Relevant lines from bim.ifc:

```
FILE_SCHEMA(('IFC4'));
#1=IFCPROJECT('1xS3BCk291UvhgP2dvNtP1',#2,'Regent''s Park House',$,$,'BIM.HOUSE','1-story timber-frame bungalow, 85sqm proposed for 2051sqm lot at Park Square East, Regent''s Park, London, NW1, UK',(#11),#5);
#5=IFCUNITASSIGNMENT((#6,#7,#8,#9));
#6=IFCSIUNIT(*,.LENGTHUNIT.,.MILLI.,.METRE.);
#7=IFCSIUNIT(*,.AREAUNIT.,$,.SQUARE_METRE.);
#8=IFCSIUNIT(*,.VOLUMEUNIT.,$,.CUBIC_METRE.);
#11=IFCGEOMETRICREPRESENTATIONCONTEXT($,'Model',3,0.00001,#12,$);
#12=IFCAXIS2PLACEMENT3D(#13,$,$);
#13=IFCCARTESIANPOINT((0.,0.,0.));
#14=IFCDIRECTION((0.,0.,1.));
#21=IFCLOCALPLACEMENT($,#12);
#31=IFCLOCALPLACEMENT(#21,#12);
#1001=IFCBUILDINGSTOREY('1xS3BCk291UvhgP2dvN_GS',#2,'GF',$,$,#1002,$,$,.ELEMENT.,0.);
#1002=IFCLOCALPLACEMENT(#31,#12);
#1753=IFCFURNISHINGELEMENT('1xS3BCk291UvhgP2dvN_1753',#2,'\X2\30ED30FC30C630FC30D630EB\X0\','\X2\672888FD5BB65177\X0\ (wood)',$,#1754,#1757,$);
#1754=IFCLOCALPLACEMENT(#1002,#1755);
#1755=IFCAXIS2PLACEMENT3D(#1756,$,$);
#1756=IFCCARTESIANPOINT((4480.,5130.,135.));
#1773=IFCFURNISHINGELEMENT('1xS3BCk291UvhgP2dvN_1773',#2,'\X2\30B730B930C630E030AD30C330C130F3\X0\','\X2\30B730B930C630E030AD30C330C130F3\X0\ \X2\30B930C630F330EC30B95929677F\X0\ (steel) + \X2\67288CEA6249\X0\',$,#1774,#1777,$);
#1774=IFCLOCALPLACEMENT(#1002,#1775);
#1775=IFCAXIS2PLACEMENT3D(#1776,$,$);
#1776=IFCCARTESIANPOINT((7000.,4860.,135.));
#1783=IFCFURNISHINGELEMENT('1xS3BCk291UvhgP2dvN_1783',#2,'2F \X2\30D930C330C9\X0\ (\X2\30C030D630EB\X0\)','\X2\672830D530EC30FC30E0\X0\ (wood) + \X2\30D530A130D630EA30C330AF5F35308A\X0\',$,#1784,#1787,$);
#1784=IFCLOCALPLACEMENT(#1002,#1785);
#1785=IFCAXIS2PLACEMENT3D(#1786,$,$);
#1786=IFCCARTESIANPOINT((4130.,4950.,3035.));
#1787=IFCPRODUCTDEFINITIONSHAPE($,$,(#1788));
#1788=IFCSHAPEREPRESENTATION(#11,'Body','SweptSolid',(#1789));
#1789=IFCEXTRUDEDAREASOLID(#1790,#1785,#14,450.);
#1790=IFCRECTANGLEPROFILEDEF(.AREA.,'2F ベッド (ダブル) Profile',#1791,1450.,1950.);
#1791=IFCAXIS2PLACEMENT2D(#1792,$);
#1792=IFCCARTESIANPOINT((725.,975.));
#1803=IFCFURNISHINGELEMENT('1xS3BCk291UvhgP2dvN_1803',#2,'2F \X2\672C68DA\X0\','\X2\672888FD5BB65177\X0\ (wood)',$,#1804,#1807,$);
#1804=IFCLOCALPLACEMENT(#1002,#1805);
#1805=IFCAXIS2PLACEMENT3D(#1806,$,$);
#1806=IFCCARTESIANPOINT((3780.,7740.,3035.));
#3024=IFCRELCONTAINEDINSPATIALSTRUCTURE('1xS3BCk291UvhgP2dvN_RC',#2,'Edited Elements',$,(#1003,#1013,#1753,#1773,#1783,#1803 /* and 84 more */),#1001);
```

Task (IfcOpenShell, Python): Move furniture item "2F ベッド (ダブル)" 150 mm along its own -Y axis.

```python
import ifcopenshell
import ifcopenshell.api.geometry
import ifcopenshell.util.placement
import ifcopenshell.util.unit

model = ifcopenshell.open("bim.ifc")
unit_scale = ifcopenshell.util.unit.calculate_unit_scale(model)

item = model.by_guid("1xS3BCk291UvhgP2dvN_1783")
matrix = ifcopenshell.util.placement.get_local_placement(item.ObjectPlacement)
matrix[:3, 3] -= matrix[:3, 1] * 0.15 / unit_scale
ifcopenshell.api.geometry.edit_object_placement(model, product=item, matrix=matrix, is_si=False)

print(ifcopenshell.util.placement.get_local_placement(item.ObjectPlacement).round(3) + 0.0)

model.write("bim_v2.ifc")
```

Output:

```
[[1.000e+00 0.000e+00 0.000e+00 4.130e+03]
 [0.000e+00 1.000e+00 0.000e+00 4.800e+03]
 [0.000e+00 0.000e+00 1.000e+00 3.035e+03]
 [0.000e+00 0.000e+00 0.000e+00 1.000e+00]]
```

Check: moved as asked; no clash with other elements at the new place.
